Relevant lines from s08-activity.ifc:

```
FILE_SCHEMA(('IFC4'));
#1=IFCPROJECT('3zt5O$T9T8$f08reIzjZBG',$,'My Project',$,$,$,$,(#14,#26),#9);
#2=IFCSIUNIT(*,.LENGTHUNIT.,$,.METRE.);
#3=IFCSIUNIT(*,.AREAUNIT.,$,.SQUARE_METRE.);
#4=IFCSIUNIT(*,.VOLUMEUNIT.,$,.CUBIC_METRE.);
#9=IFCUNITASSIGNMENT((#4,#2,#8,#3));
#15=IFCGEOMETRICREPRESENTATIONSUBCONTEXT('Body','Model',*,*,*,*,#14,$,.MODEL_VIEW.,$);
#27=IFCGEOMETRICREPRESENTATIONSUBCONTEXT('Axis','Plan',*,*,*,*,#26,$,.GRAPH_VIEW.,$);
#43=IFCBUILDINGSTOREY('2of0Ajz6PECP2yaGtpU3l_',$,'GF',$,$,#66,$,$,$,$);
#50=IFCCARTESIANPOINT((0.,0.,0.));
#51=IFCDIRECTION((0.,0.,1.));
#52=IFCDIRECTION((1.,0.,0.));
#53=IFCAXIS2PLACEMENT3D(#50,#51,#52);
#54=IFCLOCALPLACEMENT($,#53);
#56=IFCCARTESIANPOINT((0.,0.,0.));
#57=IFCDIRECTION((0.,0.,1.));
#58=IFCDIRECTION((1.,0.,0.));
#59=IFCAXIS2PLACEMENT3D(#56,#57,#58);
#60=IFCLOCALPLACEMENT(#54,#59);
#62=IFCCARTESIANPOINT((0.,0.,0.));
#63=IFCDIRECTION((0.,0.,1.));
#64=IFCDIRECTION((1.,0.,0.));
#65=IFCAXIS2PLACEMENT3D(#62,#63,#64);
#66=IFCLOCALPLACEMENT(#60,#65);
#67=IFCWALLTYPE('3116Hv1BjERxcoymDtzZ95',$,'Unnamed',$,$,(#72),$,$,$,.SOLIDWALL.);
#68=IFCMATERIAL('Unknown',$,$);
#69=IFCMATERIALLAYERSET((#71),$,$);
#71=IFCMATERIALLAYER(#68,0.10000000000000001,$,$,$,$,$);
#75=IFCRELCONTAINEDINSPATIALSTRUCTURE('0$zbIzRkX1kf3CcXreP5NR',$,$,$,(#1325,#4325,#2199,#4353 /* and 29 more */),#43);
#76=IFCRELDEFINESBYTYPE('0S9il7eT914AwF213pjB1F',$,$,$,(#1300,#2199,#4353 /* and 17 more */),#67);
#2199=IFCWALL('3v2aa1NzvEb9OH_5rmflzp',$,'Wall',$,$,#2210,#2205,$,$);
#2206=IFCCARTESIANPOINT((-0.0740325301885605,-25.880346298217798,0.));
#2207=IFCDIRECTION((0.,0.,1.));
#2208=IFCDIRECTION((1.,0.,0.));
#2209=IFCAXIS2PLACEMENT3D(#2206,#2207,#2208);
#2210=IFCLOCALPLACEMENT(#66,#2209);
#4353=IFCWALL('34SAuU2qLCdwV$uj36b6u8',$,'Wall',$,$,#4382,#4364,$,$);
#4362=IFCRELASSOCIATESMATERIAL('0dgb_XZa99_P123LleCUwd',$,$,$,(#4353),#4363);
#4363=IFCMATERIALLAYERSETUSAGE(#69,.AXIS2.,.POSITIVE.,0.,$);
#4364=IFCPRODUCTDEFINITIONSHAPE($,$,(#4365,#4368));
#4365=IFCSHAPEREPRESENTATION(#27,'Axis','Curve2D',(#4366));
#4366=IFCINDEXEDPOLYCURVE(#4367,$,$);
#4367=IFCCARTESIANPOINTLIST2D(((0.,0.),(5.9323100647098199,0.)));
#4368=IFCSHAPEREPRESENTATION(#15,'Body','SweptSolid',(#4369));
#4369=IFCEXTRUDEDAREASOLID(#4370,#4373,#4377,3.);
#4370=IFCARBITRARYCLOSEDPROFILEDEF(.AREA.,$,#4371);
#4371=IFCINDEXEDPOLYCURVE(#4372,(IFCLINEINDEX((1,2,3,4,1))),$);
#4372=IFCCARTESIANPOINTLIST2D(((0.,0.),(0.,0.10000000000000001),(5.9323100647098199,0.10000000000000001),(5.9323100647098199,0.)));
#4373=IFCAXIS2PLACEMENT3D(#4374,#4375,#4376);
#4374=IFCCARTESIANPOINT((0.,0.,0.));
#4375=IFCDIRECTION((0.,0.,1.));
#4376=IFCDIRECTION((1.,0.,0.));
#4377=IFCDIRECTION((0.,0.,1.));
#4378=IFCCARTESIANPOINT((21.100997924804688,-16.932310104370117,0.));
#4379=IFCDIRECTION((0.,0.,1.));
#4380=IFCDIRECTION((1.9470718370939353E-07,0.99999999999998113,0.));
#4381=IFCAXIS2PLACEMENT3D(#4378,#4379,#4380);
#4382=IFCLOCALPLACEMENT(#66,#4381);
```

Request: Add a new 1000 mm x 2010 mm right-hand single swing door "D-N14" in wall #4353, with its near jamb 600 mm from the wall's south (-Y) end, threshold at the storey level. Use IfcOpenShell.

```python
import numpy as np
import ifcopenshell
import ifcopenshell.api.feature
import ifcopenshell.api.geometry
import ifcopenshell.api.root
import ifcopenshell.api.spatial
import ifcopenshell.geom
import ifcopenshell.util.element
import ifcopenshell.util.placement
import ifcopenshell.util.representation
import ifcopenshell.util.shape
import ifcopenshell.util.unit

model = ifcopenshell.open("s08-activity.ifc")
unit_scale = ifcopenshell.util.unit.calculate_unit_scale(model)
settings = ifcopenshell.geom.settings()


def volume(element):
    """Net volume in cubic metres, openings subtracted."""
    shape = ifcopenshell.geom.create_shape(settings, element)
    return ifcopenshell.util.shape.get_volume(shape.geometry)


wall = model.by_id(4353)
storey = ifcopenshell.util.element.get_container(wall, ifc_class="IfcBuildingStorey")
context = ifcopenshell.util.representation.get_context(model, "Model", "Body", "MODEL_VIEW")
before = volume(wall)

width, height, from_end, sill = 1, 2.01, 0.6, 0.0  # metres

# The wall runs along its own X axis, and the end named is its -X end.
wall_shape = ifcopenshell.geom.create_shape(settings, wall)
x, y, z = ifcopenshell.util.shape.get_vertices(wall_shape.geometry).T
start = x.min() + from_end
face, thickness = float(y.min()), float(y.max() - y.min())
wall_matrix = ifcopenshell.util.placement.get_local_placement(wall.ObjectPlacement)
level = ifcopenshell.util.placement.get_local_placement(storey.ObjectPlacement)[2, 3]


def in_wall(x, y):
    """Placement at x, y metres in the wall's axes, at sill height."""
    matrix = wall_matrix.copy()
    matrix[:, 3] = wall_matrix @ np.array([x / unit_scale, y / unit_scale, 0.0, 1.0])
    matrix[2, 3] = level + sill / unit_scale
    return matrix


# Opening: a box that overshoots both wall faces by 50 mm.
opening = ifcopenshell.api.root.create_entity(model, ifc_class="IfcOpeningElement", predefined_type="OPENING")
box = ifcopenshell.api.geometry.add_wall_representation(
    model, context=context, length=width, height=height, thickness=thickness + 0.1
)
ifcopenshell.api.geometry.assign_representation(model, product=opening, representation=box)
ifcopenshell.api.geometry.edit_object_placement(model, product=opening, matrix=in_wall(start, face - 0.05), is_si=False)
ifcopenshell.api.feature.add_feature(model, feature=opening, element=wall)

door = ifcopenshell.api.root.create_entity(model, ifc_class="IfcDoor", name="D-N14", predefined_type="DOOR")
door.OverallWidth, door.OverallHeight = width / unit_scale, height / unit_scale
door.OperationType = "SINGLE_SWING_RIGHT"
body = ifcopenshell.api.geometry.add_door_representation(
    model,
    context=context,
    overall_width=door.OverallWidth,
    overall_height=door.OverallHeight,
    operation_type="SINGLE_SWING_RIGHT",
    lining_properties={"LiningDepth": thickness / unit_scale, "ThresholdDepth": thickness / unit_scale},
)
ifcopenshell.api.geometry.assign_representation(model, product=door, representation=body)
ifcopenshell.api.spatial.assign_container(model, products=[door], relating_structure=storey)
ifcopenshell.api.feature.add_filling(model, opening=opening, element=door)

# The lining spans the wall, so the door starts at the wall face.
ifcopenshell.api.geometry.edit_object_placement(model, product=door, matrix=in_wall(start, face), is_si=False)

after = volume(wall)

print(f"wall volume {before:.3f} -> {after:.3f} m3")

model.write("s08-activity-out.ifc")
```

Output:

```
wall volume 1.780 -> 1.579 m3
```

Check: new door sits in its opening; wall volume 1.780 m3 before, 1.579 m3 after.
